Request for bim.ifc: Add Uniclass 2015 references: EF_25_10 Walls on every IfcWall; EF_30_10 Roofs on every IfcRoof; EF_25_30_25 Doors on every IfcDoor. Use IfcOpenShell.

First a look at what the model holds.

```python
import ifcopenshell

model = ifcopenshell.open("bim.ifc")
print(model.schema)
print("classifications:", [c.Name for c in model.by_type("IfcClassification")])
for ifc_class in ("IfcDoor", "IfcRoof", "IfcStair", "IfcWall", "IfcWindow"):
    print(ifc_class, len(model.by_type(ifc_class)))
```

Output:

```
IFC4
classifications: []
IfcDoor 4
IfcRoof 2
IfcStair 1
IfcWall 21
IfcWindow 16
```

```python
import ifcopenshell
import ifcopenshell.api.classification

model = ifcopenshell.open("bim.ifc")

system = ifcopenshell.api.classification.add_classification(model, classification="Uniclass 2015")

codes = {
    "IfcWall": ("EF_25_10", "Walls"),
    "IfcRoof": ("EF_30_10", "Roofs"),
    "IfcDoor": ("EF_25_30_25", "Doors"),
}
for ifc_class, (code, name) in codes.items():
    products = model.by_type(ifc_class)
    ifcopenshell.api.classification.add_reference(
        model, products=products, classification=system, identification=code, name=name
    )
    print(code, len(products))

model.write("bim_edited.ifc")
```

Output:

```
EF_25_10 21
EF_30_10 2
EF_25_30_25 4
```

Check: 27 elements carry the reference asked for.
